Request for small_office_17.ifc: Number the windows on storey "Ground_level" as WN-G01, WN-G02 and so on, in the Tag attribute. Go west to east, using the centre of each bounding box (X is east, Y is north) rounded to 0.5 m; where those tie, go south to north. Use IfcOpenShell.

First a look at what the model holds.

```python
import ifcopenshell
import ifcopenshell.util.element
import ifcopenshell.util.placement

model = ifcopenshell.open("small_office_17.ifc")
print(model.schema)
storey = next(s for s in model.by_type("IfcBuildingStorey") if s.Name == "Ground_level")
windows = [e for e in ifcopenshell.util.element.get_decomposition(storey) if e.is_a("IfcWindow")]
for e in sorted(windows, key=lambda e: e.id()):
    origin = ifcopenshell.util.placement.get_local_placement(e.ObjectPlacement)[:3, 3]
    print(e.id(), e.Tag, e.Name, origin.round(2) + 0.0, sep=" | ")
```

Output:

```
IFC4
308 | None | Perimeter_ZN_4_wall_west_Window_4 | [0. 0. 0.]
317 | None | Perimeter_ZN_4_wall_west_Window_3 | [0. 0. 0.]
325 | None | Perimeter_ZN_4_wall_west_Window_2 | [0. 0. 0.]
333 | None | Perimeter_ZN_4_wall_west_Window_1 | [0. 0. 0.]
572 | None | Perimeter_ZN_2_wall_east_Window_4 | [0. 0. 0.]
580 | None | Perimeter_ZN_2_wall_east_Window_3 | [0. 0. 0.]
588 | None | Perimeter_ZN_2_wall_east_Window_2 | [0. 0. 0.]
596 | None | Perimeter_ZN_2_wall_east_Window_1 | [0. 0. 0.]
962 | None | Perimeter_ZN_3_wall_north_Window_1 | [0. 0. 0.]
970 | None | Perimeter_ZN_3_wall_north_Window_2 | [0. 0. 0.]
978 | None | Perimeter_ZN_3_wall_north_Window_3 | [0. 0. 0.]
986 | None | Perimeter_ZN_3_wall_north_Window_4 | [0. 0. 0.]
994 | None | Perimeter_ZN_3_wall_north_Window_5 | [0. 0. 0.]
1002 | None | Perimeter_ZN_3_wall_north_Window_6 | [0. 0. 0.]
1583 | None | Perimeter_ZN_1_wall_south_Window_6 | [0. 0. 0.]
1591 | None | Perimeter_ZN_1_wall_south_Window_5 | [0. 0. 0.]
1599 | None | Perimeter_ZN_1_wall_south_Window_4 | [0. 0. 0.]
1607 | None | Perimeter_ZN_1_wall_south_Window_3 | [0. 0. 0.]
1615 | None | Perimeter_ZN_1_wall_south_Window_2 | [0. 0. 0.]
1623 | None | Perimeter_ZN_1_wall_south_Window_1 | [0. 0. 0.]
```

```python
import ifcopenshell
import ifcopenshell.geom
import ifcopenshell.util.element
import ifcopenshell.util.shape

model = ifcopenshell.open("small_office_17.ifc")
settings = ifcopenshell.geom.settings()
settings.set("use-world-coords", True)


def centre(element):
    shape = ifcopenshell.geom.create_shape(settings, element)
    return ifcopenshell.util.shape.get_bbox_centroid(shape.geometry)


storey = next(s for s in model.by_type("IfcBuildingStorey") if s.Name == "Ground_level")
windows = [e for e in ifcopenshell.util.element.get_decomposition(storey) if e.is_a("IfcWindow")]

# Insertion points can sit at a corner or the storey origin, so sort by the geometry (in metres).
centres = {e: centre(e) for e in windows}
windows.sort(key=lambda e: (round(centres[e][0] / 0.5), centres[e][1]))

for i, e in enumerate(windows, start=1):
    number = f"WN-G{i:02d}"
    e.Tag = number
    print(e.id(), number)

model.write("small_office_17-out.ifc")
```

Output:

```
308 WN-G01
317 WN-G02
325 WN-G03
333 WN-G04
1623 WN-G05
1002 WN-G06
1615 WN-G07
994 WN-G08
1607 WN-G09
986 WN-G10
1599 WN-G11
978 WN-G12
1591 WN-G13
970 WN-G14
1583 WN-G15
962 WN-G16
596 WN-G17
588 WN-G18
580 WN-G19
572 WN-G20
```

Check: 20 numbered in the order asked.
